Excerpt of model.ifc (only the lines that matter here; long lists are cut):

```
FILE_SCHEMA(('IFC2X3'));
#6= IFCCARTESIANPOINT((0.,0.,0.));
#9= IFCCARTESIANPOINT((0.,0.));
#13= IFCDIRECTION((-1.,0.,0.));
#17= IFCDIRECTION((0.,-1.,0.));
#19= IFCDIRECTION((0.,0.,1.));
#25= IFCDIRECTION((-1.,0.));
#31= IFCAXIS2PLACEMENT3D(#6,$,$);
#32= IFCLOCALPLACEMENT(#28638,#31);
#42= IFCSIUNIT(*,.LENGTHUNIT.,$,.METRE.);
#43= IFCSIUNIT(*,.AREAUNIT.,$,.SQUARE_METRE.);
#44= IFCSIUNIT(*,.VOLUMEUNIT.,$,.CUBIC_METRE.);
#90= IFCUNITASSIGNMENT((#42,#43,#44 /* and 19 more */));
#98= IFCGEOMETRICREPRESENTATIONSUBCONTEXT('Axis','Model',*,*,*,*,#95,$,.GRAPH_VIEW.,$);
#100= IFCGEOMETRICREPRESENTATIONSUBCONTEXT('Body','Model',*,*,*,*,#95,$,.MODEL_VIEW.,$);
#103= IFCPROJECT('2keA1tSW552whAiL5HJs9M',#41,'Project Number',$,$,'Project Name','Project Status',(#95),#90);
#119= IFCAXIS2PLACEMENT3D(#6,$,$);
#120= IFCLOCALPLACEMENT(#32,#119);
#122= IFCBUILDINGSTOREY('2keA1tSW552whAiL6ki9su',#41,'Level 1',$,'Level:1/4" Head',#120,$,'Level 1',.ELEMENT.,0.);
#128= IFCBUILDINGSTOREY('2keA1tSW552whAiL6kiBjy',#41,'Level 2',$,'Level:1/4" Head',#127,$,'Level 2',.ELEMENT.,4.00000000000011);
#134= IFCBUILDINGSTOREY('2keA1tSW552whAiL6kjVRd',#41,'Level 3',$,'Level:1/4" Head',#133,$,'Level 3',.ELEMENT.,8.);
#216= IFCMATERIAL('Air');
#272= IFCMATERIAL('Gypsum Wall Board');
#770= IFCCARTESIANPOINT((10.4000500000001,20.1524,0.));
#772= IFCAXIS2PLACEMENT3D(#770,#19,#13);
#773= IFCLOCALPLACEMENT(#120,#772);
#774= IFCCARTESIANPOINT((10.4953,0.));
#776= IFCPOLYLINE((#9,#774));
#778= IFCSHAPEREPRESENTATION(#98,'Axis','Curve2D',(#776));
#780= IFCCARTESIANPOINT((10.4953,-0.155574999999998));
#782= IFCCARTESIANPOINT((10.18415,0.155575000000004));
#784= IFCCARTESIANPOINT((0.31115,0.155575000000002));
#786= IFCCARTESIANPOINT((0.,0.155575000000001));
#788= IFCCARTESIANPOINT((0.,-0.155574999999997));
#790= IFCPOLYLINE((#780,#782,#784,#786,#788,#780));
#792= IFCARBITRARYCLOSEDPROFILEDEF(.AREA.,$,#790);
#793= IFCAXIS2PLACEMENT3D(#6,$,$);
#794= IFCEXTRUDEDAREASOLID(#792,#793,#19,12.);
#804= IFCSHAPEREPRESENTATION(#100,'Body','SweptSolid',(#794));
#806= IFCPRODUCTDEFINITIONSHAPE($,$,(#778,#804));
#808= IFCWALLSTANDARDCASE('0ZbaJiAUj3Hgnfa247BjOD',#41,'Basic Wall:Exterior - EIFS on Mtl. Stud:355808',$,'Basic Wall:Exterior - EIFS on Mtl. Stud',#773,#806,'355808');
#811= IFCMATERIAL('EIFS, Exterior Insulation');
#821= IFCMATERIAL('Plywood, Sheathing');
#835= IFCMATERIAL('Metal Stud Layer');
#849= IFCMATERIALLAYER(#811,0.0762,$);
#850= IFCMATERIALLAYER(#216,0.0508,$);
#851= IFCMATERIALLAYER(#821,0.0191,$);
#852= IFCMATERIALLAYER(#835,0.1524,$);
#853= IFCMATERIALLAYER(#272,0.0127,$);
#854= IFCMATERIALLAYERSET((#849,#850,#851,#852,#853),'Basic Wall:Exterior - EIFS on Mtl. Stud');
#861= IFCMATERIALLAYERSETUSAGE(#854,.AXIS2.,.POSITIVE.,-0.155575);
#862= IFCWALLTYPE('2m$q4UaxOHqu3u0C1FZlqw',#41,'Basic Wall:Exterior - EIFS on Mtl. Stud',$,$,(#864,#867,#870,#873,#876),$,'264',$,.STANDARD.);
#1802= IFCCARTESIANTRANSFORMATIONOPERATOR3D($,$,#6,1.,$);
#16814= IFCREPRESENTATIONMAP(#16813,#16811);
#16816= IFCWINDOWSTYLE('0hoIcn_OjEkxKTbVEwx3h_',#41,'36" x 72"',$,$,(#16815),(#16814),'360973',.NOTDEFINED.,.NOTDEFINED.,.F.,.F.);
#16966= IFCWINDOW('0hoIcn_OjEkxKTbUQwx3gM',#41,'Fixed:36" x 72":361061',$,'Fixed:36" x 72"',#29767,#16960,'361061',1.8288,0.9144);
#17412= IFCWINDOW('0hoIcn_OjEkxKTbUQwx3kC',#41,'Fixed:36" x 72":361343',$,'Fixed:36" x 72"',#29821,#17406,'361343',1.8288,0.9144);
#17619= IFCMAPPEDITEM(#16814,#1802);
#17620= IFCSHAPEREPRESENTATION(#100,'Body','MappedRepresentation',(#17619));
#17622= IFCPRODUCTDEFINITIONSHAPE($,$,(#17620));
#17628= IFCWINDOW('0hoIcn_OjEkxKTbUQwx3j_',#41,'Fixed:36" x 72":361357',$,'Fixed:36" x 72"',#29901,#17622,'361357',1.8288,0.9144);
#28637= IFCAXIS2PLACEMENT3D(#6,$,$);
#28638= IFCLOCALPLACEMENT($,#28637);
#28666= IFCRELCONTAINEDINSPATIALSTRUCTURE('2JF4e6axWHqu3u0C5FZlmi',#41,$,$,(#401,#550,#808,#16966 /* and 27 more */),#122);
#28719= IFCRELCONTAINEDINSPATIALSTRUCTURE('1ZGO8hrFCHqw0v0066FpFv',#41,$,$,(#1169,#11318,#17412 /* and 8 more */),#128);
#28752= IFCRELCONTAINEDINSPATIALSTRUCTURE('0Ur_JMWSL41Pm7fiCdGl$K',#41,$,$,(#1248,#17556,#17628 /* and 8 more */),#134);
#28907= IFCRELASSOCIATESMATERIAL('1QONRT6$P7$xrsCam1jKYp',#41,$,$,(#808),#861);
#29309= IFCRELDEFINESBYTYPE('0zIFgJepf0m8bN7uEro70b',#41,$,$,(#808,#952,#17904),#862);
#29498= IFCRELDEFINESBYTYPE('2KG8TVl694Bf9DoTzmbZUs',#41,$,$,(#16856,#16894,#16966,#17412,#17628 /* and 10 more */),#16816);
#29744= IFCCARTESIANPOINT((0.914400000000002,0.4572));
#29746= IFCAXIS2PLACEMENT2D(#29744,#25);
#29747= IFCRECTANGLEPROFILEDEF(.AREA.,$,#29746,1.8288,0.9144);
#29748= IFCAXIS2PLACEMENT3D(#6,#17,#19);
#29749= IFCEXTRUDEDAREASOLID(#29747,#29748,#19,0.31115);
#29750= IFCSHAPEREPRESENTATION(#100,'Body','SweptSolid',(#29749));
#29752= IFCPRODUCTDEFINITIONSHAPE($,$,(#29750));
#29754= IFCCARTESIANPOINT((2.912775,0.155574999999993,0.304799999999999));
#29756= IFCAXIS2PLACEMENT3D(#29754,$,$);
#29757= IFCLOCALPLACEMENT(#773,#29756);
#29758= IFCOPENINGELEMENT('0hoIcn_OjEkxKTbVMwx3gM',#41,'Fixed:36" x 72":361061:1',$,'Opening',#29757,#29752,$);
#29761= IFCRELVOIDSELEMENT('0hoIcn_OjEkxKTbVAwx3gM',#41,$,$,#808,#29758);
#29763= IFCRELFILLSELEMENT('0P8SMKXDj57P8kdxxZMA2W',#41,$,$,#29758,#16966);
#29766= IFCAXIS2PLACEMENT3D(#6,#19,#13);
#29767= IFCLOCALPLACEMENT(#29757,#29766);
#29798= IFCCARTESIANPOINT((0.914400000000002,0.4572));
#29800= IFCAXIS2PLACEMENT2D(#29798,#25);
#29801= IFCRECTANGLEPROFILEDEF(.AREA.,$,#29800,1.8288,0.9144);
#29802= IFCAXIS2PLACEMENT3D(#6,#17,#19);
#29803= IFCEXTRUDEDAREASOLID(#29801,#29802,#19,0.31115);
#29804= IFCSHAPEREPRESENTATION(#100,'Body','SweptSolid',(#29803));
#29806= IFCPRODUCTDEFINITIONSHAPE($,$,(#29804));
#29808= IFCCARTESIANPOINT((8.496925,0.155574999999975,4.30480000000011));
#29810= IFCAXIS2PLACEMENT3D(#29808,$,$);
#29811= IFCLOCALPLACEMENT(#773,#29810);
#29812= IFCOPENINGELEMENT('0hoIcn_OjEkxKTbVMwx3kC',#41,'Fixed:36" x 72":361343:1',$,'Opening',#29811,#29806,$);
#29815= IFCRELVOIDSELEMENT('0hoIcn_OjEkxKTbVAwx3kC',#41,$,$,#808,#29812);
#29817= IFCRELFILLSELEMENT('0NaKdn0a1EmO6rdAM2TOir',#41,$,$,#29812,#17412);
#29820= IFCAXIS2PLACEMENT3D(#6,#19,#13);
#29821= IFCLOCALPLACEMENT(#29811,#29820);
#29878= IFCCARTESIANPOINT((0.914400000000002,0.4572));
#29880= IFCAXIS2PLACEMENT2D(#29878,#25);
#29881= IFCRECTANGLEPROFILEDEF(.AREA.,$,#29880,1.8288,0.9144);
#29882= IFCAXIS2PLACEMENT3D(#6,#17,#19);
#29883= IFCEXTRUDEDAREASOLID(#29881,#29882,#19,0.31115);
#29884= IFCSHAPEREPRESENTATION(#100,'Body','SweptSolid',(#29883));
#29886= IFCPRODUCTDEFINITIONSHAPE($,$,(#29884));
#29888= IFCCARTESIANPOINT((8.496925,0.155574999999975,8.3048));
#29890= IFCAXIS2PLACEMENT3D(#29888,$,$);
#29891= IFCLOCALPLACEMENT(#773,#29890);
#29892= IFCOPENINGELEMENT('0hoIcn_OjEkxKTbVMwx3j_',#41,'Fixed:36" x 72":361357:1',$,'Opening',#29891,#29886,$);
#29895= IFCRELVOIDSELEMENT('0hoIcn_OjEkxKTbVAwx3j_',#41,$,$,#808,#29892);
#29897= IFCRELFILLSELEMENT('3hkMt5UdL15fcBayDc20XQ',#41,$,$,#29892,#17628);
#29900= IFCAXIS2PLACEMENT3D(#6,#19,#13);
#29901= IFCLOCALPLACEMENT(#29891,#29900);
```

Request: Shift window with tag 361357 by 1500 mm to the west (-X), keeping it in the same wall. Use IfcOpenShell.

```python
import ifcopenshell
import ifcopenshell.api.geometry
import ifcopenshell.util.placement

model = ifcopenshell.open("model.ifc")

window = model.by_id(17628)
opening = window.FillsVoids[0].RelatingOpeningElement
wall = opening.VoidsElements[0].RelatingBuildingElement

wall_matrix = ifcopenshell.util.placement.get_local_placement(wall.ObjectPlacement)
shift = wall_matrix[:3, 0] * 1.5
before = ifcopenshell.util.placement.get_local_placement(window.ObjectPlacement)[:3, 3].copy()

# The window is placed relative to its opening, so it follows when the opening moves.
matrix = ifcopenshell.util.placement.get_local_placement(opening.ObjectPlacement)
matrix[:3, 3] += shift
ifcopenshell.api.geometry.edit_object_placement(
    model, product=opening, matrix=matrix, is_si=False, should_transform_children=True
)

after = ifcopenshell.util.placement.get_local_placement(window.ObjectPlacement)[:3, 3]
print("window moved by", (after - before).round(3) + 0.0)

model.write("model-out.ifc")
```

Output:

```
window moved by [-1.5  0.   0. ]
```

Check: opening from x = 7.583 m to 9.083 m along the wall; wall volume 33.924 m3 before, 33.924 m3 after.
